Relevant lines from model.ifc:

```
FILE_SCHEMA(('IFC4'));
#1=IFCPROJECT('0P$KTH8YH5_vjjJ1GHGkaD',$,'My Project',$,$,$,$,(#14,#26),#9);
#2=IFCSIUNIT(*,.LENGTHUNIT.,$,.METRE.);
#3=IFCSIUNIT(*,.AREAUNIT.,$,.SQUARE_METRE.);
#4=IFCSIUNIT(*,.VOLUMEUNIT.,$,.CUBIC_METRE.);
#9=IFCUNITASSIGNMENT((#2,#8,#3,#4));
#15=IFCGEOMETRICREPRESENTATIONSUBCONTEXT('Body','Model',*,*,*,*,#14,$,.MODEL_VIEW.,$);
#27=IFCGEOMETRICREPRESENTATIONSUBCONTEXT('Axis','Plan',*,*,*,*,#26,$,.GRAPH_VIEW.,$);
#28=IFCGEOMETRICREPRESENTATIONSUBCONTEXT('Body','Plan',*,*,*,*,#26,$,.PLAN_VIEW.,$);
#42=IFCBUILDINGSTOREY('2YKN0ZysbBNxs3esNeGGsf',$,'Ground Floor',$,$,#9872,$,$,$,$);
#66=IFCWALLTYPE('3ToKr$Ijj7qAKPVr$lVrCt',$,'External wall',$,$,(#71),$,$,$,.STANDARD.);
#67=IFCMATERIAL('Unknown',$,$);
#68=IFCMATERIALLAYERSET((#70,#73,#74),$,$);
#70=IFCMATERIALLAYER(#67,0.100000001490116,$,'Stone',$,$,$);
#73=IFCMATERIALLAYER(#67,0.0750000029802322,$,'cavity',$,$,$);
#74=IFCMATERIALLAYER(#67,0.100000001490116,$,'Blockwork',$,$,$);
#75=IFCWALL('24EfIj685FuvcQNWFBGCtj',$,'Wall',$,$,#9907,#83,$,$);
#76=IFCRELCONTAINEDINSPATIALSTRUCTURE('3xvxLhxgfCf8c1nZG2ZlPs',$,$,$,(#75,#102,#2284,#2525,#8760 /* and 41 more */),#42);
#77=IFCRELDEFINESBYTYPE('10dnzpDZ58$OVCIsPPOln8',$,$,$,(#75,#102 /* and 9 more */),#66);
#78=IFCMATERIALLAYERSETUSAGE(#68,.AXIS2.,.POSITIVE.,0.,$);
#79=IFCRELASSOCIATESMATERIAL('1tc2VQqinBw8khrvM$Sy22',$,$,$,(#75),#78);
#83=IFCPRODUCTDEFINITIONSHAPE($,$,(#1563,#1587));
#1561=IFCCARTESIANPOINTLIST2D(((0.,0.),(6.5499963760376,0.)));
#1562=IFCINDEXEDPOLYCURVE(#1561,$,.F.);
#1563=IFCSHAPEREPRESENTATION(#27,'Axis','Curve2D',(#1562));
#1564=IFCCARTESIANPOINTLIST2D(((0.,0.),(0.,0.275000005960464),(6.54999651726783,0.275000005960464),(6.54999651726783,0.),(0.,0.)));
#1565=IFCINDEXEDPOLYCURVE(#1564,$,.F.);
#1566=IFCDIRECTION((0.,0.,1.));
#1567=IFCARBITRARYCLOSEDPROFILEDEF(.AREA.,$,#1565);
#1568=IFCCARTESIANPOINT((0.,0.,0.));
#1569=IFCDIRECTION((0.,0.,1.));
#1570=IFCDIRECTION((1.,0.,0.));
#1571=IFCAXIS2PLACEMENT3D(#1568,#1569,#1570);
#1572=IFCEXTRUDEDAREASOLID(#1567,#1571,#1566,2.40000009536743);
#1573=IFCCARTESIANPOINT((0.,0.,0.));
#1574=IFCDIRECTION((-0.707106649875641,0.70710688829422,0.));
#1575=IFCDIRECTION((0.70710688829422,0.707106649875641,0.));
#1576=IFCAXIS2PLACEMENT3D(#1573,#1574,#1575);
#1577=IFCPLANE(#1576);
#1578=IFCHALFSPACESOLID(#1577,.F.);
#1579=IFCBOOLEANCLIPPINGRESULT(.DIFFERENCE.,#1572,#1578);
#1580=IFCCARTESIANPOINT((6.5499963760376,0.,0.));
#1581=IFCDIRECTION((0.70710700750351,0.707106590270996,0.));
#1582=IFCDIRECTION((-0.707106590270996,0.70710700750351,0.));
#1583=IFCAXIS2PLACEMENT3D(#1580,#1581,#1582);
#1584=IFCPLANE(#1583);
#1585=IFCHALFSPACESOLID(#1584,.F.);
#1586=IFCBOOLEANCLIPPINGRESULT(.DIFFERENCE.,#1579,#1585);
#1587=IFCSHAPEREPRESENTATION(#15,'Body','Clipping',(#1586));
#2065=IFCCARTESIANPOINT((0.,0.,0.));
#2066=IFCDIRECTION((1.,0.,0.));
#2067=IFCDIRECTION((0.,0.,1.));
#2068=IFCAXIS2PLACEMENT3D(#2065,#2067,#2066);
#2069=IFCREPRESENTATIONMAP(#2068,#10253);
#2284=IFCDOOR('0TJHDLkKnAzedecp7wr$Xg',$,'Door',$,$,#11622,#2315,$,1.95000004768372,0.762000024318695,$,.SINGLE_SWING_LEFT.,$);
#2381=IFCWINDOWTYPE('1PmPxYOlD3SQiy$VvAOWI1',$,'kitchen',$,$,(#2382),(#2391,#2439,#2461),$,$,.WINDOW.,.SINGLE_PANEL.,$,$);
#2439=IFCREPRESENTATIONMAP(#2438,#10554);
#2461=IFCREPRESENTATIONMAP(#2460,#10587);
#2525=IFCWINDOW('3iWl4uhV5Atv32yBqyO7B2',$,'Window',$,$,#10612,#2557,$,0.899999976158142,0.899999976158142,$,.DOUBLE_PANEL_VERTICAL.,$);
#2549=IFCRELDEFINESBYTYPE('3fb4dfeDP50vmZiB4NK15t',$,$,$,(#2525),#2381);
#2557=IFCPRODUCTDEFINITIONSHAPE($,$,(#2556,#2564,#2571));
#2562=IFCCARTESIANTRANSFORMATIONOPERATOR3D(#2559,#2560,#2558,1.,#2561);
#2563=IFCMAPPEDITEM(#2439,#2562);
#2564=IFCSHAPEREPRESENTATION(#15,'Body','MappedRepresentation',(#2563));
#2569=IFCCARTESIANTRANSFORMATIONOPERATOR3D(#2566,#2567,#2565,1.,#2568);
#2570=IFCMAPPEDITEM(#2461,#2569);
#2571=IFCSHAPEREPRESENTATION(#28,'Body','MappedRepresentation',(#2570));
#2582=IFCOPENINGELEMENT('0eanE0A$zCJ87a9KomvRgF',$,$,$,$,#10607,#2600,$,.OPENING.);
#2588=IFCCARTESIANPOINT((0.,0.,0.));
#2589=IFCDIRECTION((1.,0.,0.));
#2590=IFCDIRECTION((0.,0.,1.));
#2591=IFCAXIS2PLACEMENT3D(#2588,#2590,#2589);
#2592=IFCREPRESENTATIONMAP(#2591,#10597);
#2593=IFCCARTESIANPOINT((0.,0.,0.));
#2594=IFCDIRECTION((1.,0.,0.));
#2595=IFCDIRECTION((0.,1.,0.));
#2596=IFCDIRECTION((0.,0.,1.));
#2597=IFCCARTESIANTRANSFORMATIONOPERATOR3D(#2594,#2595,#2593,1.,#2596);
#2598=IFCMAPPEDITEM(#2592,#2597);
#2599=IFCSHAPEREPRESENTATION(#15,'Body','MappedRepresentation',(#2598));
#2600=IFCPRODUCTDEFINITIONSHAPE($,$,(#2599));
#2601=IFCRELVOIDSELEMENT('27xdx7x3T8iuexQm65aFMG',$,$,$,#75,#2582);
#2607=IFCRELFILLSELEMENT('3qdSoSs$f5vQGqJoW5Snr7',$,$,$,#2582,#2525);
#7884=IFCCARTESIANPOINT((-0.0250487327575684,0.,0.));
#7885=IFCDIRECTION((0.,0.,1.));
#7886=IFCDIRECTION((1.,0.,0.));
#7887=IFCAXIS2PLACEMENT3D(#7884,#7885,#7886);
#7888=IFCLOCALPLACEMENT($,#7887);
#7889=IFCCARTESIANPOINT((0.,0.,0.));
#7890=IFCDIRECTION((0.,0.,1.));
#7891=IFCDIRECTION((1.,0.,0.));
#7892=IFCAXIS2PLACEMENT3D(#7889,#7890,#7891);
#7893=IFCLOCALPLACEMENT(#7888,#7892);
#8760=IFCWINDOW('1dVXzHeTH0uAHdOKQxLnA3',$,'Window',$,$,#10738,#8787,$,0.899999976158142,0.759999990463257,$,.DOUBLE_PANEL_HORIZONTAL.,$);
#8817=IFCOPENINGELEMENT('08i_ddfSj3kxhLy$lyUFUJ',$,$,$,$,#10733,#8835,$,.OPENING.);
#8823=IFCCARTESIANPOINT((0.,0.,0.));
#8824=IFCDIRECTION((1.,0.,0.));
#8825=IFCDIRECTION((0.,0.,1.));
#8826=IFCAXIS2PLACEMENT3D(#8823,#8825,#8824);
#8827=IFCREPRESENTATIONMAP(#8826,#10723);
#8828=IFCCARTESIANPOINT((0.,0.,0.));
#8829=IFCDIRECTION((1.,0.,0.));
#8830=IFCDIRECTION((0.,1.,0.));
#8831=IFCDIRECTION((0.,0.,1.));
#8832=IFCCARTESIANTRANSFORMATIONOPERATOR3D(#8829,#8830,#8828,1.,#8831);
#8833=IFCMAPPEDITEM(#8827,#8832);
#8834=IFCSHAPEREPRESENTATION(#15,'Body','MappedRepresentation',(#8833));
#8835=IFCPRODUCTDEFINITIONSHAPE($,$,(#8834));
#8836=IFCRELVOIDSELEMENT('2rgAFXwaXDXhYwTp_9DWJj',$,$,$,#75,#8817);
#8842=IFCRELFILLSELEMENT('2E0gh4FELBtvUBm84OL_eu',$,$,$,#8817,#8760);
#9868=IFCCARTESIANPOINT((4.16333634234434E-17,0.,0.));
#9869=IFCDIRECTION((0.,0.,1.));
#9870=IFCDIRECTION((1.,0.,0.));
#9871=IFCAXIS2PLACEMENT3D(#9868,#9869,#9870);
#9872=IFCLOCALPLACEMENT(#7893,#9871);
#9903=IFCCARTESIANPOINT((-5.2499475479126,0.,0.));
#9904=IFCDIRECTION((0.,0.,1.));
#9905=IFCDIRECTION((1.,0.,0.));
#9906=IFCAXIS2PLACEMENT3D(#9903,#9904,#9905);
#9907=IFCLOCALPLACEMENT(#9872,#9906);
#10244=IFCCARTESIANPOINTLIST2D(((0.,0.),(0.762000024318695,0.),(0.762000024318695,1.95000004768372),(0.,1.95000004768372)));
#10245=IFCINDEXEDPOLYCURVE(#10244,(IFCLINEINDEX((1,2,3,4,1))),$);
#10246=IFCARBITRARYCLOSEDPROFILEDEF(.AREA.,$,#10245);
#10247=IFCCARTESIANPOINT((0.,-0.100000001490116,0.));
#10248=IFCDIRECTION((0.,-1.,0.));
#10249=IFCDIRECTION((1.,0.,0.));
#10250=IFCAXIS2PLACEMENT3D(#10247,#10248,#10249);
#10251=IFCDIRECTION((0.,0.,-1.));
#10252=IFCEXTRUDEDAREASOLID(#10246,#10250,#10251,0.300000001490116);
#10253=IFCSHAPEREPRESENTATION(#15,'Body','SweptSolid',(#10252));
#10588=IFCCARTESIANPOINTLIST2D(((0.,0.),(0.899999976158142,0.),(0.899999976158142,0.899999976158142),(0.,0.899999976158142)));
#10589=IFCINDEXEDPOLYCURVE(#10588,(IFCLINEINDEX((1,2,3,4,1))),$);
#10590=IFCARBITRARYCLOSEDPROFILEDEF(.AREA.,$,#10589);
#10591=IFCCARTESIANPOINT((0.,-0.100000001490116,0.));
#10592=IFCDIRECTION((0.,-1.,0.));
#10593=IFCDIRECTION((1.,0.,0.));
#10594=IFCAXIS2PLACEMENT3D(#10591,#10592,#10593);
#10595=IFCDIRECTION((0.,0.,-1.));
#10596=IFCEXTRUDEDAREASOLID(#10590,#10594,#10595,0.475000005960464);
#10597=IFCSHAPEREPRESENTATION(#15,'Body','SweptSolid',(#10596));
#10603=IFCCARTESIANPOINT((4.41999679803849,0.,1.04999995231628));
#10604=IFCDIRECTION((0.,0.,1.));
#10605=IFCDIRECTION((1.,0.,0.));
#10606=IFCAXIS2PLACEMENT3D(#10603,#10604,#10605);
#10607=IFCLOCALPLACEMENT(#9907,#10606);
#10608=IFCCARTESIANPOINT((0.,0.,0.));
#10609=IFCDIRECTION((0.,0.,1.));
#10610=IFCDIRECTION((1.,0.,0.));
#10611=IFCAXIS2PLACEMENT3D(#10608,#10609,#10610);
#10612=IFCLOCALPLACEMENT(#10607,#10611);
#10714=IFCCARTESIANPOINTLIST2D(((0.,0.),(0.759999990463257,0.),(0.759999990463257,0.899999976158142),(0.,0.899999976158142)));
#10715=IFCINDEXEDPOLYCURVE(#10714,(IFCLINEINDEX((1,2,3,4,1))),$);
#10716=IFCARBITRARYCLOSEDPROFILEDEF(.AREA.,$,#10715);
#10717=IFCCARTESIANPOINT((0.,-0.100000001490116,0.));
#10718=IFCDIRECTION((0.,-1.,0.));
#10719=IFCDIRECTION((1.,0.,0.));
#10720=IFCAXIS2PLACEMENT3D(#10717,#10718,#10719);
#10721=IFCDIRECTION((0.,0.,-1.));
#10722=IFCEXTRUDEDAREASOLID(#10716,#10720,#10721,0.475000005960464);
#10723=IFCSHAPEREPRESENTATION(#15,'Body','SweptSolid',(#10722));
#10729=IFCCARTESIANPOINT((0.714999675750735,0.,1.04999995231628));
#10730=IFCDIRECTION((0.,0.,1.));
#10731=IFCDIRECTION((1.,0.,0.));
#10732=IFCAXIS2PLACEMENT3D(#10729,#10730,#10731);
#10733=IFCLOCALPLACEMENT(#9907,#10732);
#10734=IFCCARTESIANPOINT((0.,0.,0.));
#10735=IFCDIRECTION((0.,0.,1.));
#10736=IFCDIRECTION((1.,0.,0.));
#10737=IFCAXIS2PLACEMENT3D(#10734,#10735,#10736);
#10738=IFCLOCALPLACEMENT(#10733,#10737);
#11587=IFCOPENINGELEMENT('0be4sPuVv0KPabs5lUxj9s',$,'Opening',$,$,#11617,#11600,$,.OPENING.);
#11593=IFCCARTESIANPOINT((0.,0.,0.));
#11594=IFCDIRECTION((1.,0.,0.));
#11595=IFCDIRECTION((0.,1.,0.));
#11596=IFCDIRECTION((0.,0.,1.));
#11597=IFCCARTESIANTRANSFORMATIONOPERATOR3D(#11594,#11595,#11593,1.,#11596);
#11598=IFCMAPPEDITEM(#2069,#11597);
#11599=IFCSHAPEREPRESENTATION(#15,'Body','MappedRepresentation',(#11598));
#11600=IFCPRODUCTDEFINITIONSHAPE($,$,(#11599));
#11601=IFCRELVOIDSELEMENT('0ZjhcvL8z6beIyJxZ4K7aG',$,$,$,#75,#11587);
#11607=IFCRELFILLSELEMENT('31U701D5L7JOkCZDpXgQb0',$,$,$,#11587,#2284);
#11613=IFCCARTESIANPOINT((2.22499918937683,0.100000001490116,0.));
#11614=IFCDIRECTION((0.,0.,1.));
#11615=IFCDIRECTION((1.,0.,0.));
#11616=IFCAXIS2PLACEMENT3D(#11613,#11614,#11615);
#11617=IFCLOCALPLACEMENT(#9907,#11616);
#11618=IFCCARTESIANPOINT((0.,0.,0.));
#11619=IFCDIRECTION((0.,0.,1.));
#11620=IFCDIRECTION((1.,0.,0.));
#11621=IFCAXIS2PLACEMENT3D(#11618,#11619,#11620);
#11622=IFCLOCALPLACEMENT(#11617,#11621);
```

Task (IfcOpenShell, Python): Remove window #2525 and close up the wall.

```python
import ifcopenshell
import ifcopenshell.api.feature
import ifcopenshell.api.root
import ifcopenshell.geom
import ifcopenshell.util.shape

model = ifcopenshell.open("model.ifc")
settings = ifcopenshell.geom.settings()


def volume(element):
    """Net volume in cubic metres, openings subtracted."""
    shape = ifcopenshell.geom.create_shape(settings, element)
    return ifcopenshell.util.shape.get_volume(shape.geometry)


window = model.by_guid("3iWl4uhV5Atv32yBqyO7B2")
opening = window.FillsVoids[0].RelatingOpeningElement
wall = opening.VoidsElements[0].RelatingBuildingElement
before = volume(wall)

ifcopenshell.api.root.remove_product(model, product=window)
ifcopenshell.api.feature.remove_feature(model, feature=opening)

after = volume(wall)

print(f"wall volume {before:.3f} -> {after:.3f} m3")

model.write("model_rev.ifc")
```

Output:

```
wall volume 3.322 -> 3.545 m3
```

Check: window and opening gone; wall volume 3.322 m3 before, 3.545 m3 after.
